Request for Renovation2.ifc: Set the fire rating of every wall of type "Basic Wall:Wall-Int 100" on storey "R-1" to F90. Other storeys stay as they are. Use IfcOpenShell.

First a look at what the model holds.

```python
import ifcopenshell
import ifcopenshell.util.element

model = ifcopenshell.open("Renovation2.ifc")
print(model.schema)
storey = next(s for s in model.by_type("IfcBuildingStorey") if s.Name == "R-1")
walls = [e for e in ifcopenshell.util.element.get_decomposition(storey) if e.is_a("IfcWall")]
seen = {}
for e in walls:
    element_type = ifcopenshell.util.element.get_type(e)
    key = (element_type.Name if element_type != e and element_type else None, ifcopenshell.util.element.get_pset(e, "Pset_WallCommon", "FireRating"))
    seen[key] = seen.get(key, 0) + 1
for (name, value), count in sorted(seen.items(), key=str):
    print(count, "x", name, "|", value)
```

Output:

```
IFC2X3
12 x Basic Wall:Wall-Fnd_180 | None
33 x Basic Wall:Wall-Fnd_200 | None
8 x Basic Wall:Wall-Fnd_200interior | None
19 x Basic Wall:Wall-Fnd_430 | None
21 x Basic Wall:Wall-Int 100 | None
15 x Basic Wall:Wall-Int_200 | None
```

```python
import ifcopenshell
import ifcopenshell.api.pset
import ifcopenshell.util.element

model = ifcopenshell.open("Renovation2.ifc")

storey = next(s for s in model.by_type("IfcBuildingStorey") if s.Name == "R-1")
walls = [e for e in ifcopenshell.util.element.get_decomposition(storey) if e.is_a("IfcWall")]

count = 0
for e in walls:
    element_type = ifcopenshell.util.element.get_type(e)
    if element_type in (None, e) or element_type.Name != "Basic Wall:Wall-Int 100":
        continue
    # add_pset returns the element's existing set when there is one.
    pset = ifcopenshell.api.pset.add_pset(model, product=e, name="Pset_WallCommon")
    ifcopenshell.api.pset.edit_pset(model, pset=pset, properties={"FireRating": "F90"})
    count += 1

print(count, "walls updated")

model.write("Renovation2_edited.ifc")
```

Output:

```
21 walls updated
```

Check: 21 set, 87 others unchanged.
